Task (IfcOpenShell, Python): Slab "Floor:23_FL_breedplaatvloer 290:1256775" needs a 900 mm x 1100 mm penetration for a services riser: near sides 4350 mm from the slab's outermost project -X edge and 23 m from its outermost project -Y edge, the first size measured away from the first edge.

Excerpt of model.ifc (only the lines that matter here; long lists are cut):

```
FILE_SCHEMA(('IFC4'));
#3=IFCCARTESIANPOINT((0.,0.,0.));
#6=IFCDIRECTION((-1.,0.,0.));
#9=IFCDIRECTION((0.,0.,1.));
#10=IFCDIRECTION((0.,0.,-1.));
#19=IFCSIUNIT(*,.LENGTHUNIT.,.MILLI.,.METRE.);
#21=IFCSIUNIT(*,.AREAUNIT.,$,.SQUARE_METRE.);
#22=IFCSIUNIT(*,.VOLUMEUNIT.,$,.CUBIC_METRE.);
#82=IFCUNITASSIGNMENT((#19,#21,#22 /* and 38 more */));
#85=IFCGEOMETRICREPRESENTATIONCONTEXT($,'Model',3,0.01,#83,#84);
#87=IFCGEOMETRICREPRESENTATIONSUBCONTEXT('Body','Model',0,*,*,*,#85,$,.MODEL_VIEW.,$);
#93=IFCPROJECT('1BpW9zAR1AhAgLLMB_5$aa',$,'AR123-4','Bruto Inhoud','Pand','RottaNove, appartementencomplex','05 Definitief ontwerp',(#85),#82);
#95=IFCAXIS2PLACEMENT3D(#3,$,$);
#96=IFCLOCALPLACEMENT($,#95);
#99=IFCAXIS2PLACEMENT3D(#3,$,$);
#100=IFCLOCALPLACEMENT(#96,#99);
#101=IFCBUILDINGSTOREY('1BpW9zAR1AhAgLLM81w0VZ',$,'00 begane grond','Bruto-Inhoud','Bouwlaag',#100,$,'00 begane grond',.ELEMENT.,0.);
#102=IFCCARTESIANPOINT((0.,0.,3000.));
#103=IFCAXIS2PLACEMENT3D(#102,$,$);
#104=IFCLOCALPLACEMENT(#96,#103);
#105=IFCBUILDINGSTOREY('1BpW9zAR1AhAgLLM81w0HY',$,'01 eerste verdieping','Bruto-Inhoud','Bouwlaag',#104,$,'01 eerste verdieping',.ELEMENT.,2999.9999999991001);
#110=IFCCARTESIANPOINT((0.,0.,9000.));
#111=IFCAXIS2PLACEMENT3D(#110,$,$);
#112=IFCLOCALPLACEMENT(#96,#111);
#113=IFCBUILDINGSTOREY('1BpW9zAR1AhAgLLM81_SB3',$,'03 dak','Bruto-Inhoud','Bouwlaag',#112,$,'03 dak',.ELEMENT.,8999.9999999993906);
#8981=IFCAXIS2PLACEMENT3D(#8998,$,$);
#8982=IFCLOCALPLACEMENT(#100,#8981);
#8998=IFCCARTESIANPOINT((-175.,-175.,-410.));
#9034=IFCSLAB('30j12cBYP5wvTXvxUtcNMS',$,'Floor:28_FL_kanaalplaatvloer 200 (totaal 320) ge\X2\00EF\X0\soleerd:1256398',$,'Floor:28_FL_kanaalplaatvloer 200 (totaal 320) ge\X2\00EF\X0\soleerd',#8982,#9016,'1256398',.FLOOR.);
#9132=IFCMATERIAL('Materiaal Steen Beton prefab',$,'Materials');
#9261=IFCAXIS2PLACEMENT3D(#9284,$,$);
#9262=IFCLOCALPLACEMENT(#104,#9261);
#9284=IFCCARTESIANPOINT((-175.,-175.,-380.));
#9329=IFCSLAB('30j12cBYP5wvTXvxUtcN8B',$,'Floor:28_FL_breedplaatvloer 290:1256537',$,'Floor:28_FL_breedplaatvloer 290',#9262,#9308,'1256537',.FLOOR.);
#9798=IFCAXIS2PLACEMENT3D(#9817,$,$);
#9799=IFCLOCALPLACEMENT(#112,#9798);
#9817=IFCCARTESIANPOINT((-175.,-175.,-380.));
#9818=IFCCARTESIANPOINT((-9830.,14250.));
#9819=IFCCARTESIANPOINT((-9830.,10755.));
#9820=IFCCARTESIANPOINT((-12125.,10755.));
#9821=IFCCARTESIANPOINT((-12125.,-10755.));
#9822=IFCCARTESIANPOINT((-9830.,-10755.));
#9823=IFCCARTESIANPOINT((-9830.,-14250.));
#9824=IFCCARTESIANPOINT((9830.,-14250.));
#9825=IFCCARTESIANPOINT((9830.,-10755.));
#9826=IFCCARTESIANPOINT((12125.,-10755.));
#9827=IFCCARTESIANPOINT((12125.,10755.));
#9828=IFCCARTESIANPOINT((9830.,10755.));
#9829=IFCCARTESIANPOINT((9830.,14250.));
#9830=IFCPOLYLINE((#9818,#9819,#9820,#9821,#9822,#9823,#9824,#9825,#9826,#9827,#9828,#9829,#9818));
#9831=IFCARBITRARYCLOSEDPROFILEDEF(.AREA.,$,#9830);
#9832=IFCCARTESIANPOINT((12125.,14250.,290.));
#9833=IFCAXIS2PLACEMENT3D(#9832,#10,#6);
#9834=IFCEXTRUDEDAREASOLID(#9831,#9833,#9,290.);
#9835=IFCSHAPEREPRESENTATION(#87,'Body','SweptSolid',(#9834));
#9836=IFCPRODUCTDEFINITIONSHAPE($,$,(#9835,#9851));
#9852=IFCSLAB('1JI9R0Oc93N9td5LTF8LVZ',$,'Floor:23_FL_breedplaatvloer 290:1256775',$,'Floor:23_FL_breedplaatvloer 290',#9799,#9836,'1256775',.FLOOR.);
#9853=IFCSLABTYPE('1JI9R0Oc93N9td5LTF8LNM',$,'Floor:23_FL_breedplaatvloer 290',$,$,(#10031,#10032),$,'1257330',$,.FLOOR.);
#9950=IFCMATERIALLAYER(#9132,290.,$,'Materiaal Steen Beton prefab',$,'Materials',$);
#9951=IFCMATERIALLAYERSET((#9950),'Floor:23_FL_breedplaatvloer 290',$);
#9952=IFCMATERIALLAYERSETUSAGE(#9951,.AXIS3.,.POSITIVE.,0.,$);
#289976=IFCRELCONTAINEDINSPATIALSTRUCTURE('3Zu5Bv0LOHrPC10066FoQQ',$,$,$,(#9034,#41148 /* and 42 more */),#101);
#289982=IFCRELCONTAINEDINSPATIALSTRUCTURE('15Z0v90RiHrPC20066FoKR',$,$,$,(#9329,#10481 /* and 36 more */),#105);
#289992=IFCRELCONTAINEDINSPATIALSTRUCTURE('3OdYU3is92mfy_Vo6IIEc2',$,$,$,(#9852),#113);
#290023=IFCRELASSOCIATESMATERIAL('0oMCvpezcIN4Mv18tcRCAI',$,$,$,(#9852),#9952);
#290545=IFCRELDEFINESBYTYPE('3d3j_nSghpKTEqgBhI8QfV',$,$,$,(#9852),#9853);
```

```python
import numpy as np
import ifcopenshell
import ifcopenshell.api.feature
import ifcopenshell.api.geometry
import ifcopenshell.api.root
import ifcopenshell.geom
import ifcopenshell.util.placement
import ifcopenshell.util.representation
import ifcopenshell.util.shape
import ifcopenshell.util.unit

model = ifcopenshell.open("model.ifc")
unit_scale = ifcopenshell.util.unit.calculate_unit_scale(model)
settings = ifcopenshell.geom.settings()


def volume(element):
    """Net volume in cubic metres, openings subtracted."""
    shape = ifcopenshell.geom.create_shape(settings, element)
    return ifcopenshell.util.shape.get_volume(shape.geometry)


slab = model.by_id(9852)
before = volume(slab)

# Extent in the slab's own axes, in metres. The edges named are its -X and -Y sides.
slab_shape = ifcopenshell.geom.create_shape(settings, slab)
vertices = ifcopenshell.util.shape.get_vertices(slab_shape.geometry)
x_min, y_min, bottom = vertices.min(axis=0)
top = vertices[:, 2].max()

opening = ifcopenshell.api.root.create_entity(model, ifc_class="IfcOpeningElement", name="Services riser opening", predefined_type="OPENING")
context = ifcopenshell.util.representation.get_context(model, "Model", "Body", "MODEL_VIEW")
width, depth = 0.9, 1.1
outline = [(0.0, 0.0), (width, 0.0), (width, depth), (0.0, depth), (0.0, 0.0)]
# Overshoot both faces by 50 mm so the cut is clean.
shape = ifcopenshell.api.geometry.add_slab_representation(
    model, context=context, depth=top - bottom + 0.1, polyline=outline
)
ifcopenshell.api.geometry.assign_representation(model, product=opening, representation=shape)

matrix = ifcopenshell.util.placement.get_local_placement(slab.ObjectPlacement)
matrix[:, 3] = matrix @ np.append(np.array([x_min + 4.35, y_min + 23, bottom - 0.05]) / unit_scale, 1.0)
ifcopenshell.api.geometry.edit_object_placement(model, product=opening, matrix=matrix, is_si=False)
ifcopenshell.api.feature.add_feature(model, feature=opening, element=slab)

after = volume(slab)

print(f"slab volume {before:.3f} -> {after:.3f} m3")

model.write("model_updated.ifc")
```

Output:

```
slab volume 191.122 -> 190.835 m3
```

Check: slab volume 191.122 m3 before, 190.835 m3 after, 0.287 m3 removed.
